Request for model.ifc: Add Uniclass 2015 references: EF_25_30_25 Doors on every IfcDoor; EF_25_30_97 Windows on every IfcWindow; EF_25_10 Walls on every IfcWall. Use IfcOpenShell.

First a look at what the model holds.

```python
import ifcopenshell

model = ifcopenshell.open("model.ifc")
print(model.schema)
print("classifications:", [c.Name for c in model.by_type("IfcClassification")])
for ifc_class in ("IfcDoor", "IfcRoof", "IfcStair", "IfcWall", "IfcWindow"):
    print(ifc_class, len(model.by_type(ifc_class)))
```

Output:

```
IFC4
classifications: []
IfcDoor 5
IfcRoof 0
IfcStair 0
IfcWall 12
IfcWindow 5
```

```python
import ifcopenshell
import ifcopenshell.api.classification

model = ifcopenshell.open("model.ifc")

system = ifcopenshell.api.classification.add_classification(model, classification="Uniclass 2015")

codes = {
    "IfcDoor": ("EF_25_30_25", "Doors"),
    "IfcWindow": ("EF_25_30_97", "Windows"),
    "IfcWall": ("EF_25_10", "Walls"),
}
for ifc_class, (code, name) in codes.items():
    products = model.by_type(ifc_class)
    ifcopenshell.api.classification.add_reference(
        model, products=products, classification=system, identification=code, name=name
    )
    print(code, len(products))

model.write("model_rev.ifc")
```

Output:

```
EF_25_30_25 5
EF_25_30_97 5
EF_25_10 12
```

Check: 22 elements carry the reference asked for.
